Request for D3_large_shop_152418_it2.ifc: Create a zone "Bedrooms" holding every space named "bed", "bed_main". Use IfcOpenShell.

First a look at what the model holds.

```python
import ifcopenshell

model = ifcopenshell.open("D3_large_shop_152418_it2.ifc")
print(model.schema)
seen = {}
for space in model.by_type("IfcSpace"):
    seen[space.LongName] = seen.get(space.LongName, 0) + 1
for name, count in sorted(seen.items(), key=str):
    print(count, "x", name)
print("zones:", [z.Name for z in model.by_type("IfcZone")][:20])
```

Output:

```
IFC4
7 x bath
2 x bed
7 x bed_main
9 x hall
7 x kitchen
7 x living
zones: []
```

```python
import ifcopenshell
import ifcopenshell.api.group
import ifcopenshell.api.root

model = ifcopenshell.open("D3_large_shop_152418_it2.ifc")

names = {"bed", "bed_main"}
spaces = [s for s in model.by_type("IfcSpace") if s.LongName in names]

zone = ifcopenshell.api.root.create_entity(model, ifc_class="IfcZone", name="Bedrooms")
ifcopenshell.api.group.assign_group(model, products=spaces, group=zone)
print(len(spaces), "spaces in", zone.Name)

model.write("D3_large_shop_152418_it2-out.ifc")
```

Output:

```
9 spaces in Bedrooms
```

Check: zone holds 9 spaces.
